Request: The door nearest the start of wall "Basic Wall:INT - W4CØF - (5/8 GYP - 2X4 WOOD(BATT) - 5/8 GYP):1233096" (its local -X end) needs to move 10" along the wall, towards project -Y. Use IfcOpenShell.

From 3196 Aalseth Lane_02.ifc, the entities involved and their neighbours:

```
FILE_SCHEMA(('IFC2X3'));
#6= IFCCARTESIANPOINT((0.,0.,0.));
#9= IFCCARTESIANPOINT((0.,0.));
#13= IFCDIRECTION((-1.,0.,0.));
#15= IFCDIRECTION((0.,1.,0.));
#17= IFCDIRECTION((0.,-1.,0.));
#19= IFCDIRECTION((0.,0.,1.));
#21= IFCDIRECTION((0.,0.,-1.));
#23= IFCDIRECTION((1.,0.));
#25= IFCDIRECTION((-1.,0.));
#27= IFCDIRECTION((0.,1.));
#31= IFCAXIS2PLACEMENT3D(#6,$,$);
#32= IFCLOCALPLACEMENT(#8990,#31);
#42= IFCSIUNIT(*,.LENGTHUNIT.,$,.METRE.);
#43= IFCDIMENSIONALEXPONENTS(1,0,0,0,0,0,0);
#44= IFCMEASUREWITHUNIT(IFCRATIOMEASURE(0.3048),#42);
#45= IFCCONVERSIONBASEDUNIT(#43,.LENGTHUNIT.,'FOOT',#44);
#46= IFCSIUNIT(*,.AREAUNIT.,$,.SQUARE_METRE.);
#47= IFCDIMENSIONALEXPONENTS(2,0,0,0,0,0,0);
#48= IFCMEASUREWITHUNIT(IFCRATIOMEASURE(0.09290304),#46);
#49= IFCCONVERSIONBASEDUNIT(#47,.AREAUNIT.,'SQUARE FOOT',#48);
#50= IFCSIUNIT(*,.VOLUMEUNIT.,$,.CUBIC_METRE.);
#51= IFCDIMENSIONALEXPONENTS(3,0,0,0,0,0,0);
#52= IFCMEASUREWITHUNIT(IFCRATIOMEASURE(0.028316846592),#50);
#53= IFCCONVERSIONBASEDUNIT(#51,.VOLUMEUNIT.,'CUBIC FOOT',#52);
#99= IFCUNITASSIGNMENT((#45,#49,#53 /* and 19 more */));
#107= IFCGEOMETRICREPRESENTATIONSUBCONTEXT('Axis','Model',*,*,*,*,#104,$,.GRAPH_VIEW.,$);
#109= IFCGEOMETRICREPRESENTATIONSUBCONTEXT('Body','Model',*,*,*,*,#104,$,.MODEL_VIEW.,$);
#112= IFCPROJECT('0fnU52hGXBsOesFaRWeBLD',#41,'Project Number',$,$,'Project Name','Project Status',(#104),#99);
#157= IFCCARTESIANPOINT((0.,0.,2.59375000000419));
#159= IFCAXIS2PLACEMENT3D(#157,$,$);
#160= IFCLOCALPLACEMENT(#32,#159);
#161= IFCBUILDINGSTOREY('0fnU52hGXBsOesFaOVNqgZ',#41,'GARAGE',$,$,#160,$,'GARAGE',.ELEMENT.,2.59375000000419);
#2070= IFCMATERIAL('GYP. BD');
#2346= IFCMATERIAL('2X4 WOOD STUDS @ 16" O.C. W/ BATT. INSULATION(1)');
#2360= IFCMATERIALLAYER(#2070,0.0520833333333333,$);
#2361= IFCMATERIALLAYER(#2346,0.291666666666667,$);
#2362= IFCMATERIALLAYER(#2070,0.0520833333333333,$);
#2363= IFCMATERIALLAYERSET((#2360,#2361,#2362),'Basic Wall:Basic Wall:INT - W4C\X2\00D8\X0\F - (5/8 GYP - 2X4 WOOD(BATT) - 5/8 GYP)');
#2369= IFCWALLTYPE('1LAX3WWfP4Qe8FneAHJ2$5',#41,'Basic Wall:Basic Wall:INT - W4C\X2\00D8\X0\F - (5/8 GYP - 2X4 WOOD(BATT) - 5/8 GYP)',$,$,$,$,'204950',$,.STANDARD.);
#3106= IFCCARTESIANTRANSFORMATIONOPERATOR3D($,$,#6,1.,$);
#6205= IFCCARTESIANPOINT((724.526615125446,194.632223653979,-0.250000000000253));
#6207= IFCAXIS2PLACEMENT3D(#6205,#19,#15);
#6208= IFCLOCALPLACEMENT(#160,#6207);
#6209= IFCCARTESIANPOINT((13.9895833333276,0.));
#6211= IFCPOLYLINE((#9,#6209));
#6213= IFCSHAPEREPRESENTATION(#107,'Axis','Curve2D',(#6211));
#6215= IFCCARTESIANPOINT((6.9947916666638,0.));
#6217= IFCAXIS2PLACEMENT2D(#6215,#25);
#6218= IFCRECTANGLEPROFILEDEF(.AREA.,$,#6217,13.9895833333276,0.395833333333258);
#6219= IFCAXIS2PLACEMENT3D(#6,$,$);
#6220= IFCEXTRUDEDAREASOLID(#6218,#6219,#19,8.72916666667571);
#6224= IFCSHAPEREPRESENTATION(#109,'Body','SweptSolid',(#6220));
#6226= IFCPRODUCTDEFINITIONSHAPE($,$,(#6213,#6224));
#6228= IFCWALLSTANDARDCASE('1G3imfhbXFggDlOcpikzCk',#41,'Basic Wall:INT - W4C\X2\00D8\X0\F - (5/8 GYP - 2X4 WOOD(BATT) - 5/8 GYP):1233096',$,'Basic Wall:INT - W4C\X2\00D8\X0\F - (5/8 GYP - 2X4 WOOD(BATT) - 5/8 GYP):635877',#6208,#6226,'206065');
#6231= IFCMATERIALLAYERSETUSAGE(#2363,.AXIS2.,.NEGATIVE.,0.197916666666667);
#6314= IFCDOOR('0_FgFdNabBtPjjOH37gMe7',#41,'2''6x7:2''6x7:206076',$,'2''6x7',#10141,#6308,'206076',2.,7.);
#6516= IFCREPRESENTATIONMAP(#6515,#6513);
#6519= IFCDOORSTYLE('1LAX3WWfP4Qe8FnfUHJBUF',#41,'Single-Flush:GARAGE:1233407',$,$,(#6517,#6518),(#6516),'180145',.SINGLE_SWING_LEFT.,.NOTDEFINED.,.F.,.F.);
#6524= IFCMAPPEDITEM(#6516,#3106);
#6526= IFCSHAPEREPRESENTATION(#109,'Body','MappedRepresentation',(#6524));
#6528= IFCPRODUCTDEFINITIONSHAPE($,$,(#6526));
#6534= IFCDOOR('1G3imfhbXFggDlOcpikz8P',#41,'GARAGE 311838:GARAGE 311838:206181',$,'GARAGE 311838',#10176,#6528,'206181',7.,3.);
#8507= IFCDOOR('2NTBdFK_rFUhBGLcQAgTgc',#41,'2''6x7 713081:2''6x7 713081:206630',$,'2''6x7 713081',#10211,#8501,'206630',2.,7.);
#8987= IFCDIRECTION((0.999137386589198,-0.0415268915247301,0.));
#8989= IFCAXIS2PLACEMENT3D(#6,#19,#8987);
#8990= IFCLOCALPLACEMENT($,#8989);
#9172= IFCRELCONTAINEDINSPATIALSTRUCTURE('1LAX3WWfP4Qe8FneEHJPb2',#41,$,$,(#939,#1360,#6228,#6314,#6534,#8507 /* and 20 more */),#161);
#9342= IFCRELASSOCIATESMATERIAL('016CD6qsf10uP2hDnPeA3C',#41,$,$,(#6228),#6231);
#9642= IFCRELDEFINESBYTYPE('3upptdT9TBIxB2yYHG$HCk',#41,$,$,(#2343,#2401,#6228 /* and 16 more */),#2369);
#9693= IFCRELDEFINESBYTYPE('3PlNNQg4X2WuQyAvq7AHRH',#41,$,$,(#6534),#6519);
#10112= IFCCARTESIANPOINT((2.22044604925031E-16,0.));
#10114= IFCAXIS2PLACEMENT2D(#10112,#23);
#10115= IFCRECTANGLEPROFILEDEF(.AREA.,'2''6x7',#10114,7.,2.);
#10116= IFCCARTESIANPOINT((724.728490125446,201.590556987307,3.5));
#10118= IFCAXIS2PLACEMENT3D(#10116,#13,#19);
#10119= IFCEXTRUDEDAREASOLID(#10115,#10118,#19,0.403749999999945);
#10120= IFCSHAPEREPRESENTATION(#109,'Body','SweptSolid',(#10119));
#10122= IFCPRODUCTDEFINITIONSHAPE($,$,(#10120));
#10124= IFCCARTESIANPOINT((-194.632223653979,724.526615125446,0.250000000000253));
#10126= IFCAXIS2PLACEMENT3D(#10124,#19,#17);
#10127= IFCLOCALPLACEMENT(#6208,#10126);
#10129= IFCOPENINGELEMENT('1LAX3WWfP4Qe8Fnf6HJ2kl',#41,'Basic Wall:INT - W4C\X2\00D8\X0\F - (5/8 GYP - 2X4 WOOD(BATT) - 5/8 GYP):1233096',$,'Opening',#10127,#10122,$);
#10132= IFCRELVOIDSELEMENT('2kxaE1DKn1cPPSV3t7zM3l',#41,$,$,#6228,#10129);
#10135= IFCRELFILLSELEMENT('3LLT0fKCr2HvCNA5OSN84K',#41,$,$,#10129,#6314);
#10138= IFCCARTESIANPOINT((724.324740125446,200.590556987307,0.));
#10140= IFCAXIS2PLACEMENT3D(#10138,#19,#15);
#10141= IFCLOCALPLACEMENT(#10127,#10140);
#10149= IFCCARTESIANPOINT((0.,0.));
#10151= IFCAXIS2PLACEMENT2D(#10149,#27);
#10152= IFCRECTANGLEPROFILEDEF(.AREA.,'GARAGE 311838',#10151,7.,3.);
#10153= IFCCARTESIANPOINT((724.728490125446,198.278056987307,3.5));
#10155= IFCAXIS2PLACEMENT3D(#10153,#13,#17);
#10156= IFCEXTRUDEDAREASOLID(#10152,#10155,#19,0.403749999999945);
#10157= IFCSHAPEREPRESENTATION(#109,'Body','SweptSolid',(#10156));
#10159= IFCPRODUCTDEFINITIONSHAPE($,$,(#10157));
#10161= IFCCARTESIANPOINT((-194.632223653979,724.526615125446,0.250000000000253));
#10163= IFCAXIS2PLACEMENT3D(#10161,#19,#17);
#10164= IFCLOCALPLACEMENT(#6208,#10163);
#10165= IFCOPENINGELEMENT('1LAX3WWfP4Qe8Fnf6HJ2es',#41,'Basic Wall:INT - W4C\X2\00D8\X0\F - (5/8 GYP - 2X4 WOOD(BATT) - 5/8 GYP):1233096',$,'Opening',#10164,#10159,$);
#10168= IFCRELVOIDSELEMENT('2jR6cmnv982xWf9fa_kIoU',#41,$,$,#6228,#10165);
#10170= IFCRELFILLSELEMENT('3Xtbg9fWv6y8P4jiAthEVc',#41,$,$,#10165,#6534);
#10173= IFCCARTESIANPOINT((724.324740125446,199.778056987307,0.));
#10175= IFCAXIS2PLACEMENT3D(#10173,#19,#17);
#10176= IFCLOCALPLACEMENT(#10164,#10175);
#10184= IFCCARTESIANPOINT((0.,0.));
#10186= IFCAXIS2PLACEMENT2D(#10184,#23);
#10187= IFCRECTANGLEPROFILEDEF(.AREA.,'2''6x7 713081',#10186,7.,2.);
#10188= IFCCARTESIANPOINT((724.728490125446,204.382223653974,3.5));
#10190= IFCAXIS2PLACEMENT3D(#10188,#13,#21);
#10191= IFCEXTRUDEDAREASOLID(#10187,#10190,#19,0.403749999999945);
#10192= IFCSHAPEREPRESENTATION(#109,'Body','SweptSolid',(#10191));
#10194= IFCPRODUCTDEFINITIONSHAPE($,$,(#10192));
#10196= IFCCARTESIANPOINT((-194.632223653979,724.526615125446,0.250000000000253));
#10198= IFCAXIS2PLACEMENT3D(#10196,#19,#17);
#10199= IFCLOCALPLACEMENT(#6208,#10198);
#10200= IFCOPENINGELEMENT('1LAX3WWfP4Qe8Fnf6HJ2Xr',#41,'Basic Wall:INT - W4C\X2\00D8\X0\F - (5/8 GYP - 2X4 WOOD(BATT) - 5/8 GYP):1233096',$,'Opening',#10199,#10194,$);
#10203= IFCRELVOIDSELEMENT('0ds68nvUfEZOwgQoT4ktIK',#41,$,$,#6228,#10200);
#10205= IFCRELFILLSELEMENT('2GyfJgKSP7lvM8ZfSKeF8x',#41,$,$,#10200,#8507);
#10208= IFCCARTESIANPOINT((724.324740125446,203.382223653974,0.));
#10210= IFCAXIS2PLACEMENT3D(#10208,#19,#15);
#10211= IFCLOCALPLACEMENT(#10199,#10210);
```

```python
import ifcopenshell
import ifcopenshell.api.geometry
import ifcopenshell.util.placement
import ifcopenshell.util.unit

model = ifcopenshell.open("3196 Aalseth Lane_02.ifc")
unit_scale = ifcopenshell.util.unit.calculate_unit_scale(model)

door = model.by_guid("1G3imfhbXFggDlOcpikz8P")
opening = door.FillsVoids[0].RelatingOpeningElement
wall = opening.VoidsElements[0].RelatingBuildingElement

wall_matrix = ifcopenshell.util.placement.get_local_placement(wall.ObjectPlacement)
shift = wall_matrix[:3, 0] * -10 * 0.0254 / unit_scale
before = ifcopenshell.util.placement.get_local_placement(door.ObjectPlacement)[:3, 3].copy()

# The door is placed relative to its opening, so it follows when the opening moves.
matrix = ifcopenshell.util.placement.get_local_placement(opening.ObjectPlacement)
matrix[:3, 3] += shift
ifcopenshell.api.geometry.edit_object_placement(
    model, product=opening, matrix=matrix, is_si=False, should_transform_children=True
)

after = ifcopenshell.util.placement.get_local_placement(door.ObjectPlacement)[:3, 3]
print("door moved by", (after - before).round(3) + 0.0)

model.write("3196 Aalseth Lane_02_updated.ifc")
```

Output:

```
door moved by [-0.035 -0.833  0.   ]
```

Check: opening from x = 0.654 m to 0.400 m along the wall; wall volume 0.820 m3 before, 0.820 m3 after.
